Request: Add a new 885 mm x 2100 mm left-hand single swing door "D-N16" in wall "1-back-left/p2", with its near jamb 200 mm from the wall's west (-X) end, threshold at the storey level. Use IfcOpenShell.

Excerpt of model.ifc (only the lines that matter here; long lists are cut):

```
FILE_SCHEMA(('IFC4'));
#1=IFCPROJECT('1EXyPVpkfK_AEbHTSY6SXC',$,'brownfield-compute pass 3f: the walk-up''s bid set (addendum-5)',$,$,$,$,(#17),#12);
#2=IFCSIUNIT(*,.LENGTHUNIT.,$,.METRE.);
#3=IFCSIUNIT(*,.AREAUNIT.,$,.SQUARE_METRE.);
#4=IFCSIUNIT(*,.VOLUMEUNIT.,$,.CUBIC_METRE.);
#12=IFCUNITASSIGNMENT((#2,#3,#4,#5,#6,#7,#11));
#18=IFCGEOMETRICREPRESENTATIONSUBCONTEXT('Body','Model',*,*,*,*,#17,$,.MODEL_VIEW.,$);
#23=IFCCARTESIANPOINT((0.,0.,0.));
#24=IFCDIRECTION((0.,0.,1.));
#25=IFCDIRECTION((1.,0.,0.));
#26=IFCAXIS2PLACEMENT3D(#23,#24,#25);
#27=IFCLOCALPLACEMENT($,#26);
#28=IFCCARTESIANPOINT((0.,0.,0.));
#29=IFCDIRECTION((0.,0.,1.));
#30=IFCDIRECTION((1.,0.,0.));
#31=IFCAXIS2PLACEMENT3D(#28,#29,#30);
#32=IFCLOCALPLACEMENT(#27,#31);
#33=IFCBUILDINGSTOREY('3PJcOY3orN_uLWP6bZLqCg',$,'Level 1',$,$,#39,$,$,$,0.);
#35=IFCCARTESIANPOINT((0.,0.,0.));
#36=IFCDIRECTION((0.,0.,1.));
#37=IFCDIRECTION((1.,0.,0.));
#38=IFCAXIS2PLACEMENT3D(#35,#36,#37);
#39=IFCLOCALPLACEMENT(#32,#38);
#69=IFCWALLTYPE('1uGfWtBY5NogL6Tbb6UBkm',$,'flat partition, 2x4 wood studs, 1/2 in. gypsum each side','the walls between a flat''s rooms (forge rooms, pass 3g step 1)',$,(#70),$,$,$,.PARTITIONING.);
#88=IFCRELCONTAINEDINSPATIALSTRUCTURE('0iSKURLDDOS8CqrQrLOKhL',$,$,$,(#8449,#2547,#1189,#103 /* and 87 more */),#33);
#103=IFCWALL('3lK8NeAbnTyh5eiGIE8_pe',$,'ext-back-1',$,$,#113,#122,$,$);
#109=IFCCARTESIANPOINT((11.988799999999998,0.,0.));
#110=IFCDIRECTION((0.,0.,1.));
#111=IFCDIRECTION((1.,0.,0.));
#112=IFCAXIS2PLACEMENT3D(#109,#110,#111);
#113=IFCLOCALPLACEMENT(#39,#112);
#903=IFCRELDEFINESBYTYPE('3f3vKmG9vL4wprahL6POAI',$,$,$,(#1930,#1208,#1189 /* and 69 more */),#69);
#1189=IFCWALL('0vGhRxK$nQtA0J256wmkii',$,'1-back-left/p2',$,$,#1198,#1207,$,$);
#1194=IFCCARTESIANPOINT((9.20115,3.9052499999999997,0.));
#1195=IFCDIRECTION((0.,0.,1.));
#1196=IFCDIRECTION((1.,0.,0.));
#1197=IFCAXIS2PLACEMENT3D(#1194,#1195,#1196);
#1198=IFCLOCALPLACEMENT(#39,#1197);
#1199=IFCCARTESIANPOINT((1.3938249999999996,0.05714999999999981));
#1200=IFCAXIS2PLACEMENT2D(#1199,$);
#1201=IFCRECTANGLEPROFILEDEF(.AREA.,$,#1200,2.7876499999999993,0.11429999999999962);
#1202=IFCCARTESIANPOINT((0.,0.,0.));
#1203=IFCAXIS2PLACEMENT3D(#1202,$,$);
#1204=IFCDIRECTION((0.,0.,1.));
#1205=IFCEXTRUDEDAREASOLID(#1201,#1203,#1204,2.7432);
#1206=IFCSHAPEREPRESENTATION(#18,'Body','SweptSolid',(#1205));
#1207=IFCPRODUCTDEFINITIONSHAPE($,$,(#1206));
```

```python
import numpy as np
import ifcopenshell
import ifcopenshell.api.feature
import ifcopenshell.api.geometry
import ifcopenshell.api.root
import ifcopenshell.api.spatial
import ifcopenshell.geom
import ifcopenshell.util.element
import ifcopenshell.util.placement
import ifcopenshell.util.representation
import ifcopenshell.util.shape
import ifcopenshell.util.unit

model = ifcopenshell.open("model.ifc")
unit_scale = ifcopenshell.util.unit.calculate_unit_scale(model)
settings = ifcopenshell.geom.settings()


def volume(element):
    """Net volume in cubic metres, openings subtracted."""
    shape = ifcopenshell.geom.create_shape(settings, element)
    return ifcopenshell.util.shape.get_volume(shape.geometry)


wall = model.by_guid("0vGhRxK$nQtA0J256wmkii")
storey = ifcopenshell.util.element.get_container(wall, ifc_class="IfcBuildingStorey")
context = ifcopenshell.util.representation.get_context(model, "Model", "Body", "MODEL_VIEW")
before = volume(wall)

width, height, from_end, sill = 0.885, 2.1, 0.2, 0.0  # metres

# The wall runs along its own X axis, and the end named is its -X end.
wall_shape = ifcopenshell.geom.create_shape(settings, wall)
x, y, z = ifcopenshell.util.shape.get_vertices(wall_shape.geometry).T
start = x.min() + from_end
face, thickness = float(y.min()), float(y.max() - y.min())
wall_matrix = ifcopenshell.util.placement.get_local_placement(wall.ObjectPlacement)
level = ifcopenshell.util.placement.get_local_placement(storey.ObjectPlacement)[2, 3]


def in_wall(x, y):
    """Placement at x, y metres in the wall's axes, at sill height."""
    matrix = wall_matrix.copy()
    matrix[:, 3] = wall_matrix @ np.array([x / unit_scale, y / unit_scale, 0.0, 1.0])
    matrix[2, 3] = level + sill / unit_scale
    return matrix


# Opening: a box that overshoots both wall faces by 50 mm.
opening = ifcopenshell.api.root.create_entity(model, ifc_class="IfcOpeningElement", predefined_type="OPENING")
box = ifcopenshell.api.geometry.add_wall_representation(
    model, context=context, length=width, height=height, thickness=thickness + 0.1
)
ifcopenshell.api.geometry.assign_representation(model, product=opening, representation=box)
ifcopenshell.api.geometry.edit_object_placement(model, product=opening, matrix=in_wall(start, face - 0.05), is_si=False)
ifcopenshell.api.feature.add_feature(model, feature=opening, element=wall)

door = ifcopenshell.api.root.create_entity(model, ifc_class="IfcDoor", name="D-N16", predefined_type="DOOR")
door.OverallWidth, door.OverallHeight = width / unit_scale, height / unit_scale
door.OperationType = "SINGLE_SWING_LEFT"
body = ifcopenshell.api.geometry.add_door_representation(
    model,
    context=context,
    overall_width=door.OverallWidth,
    overall_height=door.OverallHeight,
    operation_type="SINGLE_SWING_LEFT",
    lining_properties={"LiningDepth": thickness / unit_scale, "ThresholdDepth": thickness / unit_scale},
)
ifcopenshell.api.geometry.assign_representation(model, product=door, representation=body)
ifcopenshell.api.spatial.assign_container(model, products=[door], relating_structure=storey)
ifcopenshell.api.feature.add_filling(model, opening=opening, element=door)

# The lining spans the wall, so the door starts at the wall face.
ifcopenshell.api.geometry.edit_object_placement(model, product=door, matrix=in_wall(start, face), is_si=False)

after = volume(wall)

print(f"wall volume {before:.3f} -> {after:.3f} m3")

model.write("model_edited.ifc")
```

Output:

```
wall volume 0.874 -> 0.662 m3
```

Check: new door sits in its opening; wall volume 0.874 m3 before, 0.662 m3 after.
